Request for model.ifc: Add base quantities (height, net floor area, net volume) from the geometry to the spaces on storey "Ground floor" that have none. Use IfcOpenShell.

First a look at what the model holds.

```python
import ifcopenshell
import ifcopenshell.util.element
import ifcopenshell.util.unit

model = ifcopenshell.open("model.ifc")
print(model.schema)
for unit_type in ("LENGTHUNIT", "AREAUNIT", "VOLUMEUNIT"):
    print(unit_type, ifcopenshell.util.unit.calculate_unit_scale(model, unit_type))
storey = next(s for s in model.by_type("IfcBuildingStorey") if s.Name == "Ground floor")
spaces = [e for e in ifcopenshell.util.element.get_decomposition(storey) if e.is_a("IfcSpace")]
for e in sorted(spaces, key=lambda e: e.id()):
    print(e.id(), e.is_a(), e.Name, list(ifcopenshell.util.element.get_psets(e, qtos_only=True)), sep=" | ")
```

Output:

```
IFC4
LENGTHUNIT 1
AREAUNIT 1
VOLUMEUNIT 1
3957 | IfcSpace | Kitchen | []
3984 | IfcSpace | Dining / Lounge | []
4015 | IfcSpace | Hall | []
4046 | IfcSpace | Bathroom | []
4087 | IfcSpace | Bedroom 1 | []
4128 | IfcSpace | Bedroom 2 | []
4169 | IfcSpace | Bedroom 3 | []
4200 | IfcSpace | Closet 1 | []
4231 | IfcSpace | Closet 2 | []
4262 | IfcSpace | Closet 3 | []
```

```python
import ifcopenshell
import ifcopenshell.api.pset
import ifcopenshell.geom
import ifcopenshell.util.element
import ifcopenshell.util.shape
import ifcopenshell.util.unit

model = ifcopenshell.open("model.ifc")
unit_scale = ifcopenshell.util.unit.calculate_unit_scale(model)
area_scale = ifcopenshell.util.unit.calculate_unit_scale(model, "AREAUNIT")
volume_scale = ifcopenshell.util.unit.calculate_unit_scale(model, "VOLUMEUNIT")
settings = ifcopenshell.geom.settings()

storey = next(s for s in model.by_type("IfcBuildingStorey") if s.Name == "Ground floor")
spaces = [e for e in ifcopenshell.util.element.get_decomposition(storey) if e.is_a("IfcSpace")]

for e in sorted(spaces, key=lambda e: e.id()):
    if ifcopenshell.util.element.get_psets(e, qtos_only=True, should_inherit=False):
        continue
    # Geometry comes back in metres, in the element's own axes.
    shape = ifcopenshell.geom.create_shape(settings, e)
    values = {
        "Height": ifcopenshell.util.shape.get_z(shape.geometry) / unit_scale,
        "NetFloorArea": ifcopenshell.util.shape.get_footprint_area(shape.geometry) / area_scale,
        "NetVolume": ifcopenshell.util.shape.get_volume(shape.geometry) / volume_scale,
    }
    qto = ifcopenshell.api.pset.add_qto(model, product=e, name="Qto_SpaceBaseQuantities")
    ifcopenshell.api.pset.edit_qto(model, qto=qto, properties=values)
    print(e.id(), {k: round(v, 3) for k, v in values.items()})

model.write("model_edited.ifc")
```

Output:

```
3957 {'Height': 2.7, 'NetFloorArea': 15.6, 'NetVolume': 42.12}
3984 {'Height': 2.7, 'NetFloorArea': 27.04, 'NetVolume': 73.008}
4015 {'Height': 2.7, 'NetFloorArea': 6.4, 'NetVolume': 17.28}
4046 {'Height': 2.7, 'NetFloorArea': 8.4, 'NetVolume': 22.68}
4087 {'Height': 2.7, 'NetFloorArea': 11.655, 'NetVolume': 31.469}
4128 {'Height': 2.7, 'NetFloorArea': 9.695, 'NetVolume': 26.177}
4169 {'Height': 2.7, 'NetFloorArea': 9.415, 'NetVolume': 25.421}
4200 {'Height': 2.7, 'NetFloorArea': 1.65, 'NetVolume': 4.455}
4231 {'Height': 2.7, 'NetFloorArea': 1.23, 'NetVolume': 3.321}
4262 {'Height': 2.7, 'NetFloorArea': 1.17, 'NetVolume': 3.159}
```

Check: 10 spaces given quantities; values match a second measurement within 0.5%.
